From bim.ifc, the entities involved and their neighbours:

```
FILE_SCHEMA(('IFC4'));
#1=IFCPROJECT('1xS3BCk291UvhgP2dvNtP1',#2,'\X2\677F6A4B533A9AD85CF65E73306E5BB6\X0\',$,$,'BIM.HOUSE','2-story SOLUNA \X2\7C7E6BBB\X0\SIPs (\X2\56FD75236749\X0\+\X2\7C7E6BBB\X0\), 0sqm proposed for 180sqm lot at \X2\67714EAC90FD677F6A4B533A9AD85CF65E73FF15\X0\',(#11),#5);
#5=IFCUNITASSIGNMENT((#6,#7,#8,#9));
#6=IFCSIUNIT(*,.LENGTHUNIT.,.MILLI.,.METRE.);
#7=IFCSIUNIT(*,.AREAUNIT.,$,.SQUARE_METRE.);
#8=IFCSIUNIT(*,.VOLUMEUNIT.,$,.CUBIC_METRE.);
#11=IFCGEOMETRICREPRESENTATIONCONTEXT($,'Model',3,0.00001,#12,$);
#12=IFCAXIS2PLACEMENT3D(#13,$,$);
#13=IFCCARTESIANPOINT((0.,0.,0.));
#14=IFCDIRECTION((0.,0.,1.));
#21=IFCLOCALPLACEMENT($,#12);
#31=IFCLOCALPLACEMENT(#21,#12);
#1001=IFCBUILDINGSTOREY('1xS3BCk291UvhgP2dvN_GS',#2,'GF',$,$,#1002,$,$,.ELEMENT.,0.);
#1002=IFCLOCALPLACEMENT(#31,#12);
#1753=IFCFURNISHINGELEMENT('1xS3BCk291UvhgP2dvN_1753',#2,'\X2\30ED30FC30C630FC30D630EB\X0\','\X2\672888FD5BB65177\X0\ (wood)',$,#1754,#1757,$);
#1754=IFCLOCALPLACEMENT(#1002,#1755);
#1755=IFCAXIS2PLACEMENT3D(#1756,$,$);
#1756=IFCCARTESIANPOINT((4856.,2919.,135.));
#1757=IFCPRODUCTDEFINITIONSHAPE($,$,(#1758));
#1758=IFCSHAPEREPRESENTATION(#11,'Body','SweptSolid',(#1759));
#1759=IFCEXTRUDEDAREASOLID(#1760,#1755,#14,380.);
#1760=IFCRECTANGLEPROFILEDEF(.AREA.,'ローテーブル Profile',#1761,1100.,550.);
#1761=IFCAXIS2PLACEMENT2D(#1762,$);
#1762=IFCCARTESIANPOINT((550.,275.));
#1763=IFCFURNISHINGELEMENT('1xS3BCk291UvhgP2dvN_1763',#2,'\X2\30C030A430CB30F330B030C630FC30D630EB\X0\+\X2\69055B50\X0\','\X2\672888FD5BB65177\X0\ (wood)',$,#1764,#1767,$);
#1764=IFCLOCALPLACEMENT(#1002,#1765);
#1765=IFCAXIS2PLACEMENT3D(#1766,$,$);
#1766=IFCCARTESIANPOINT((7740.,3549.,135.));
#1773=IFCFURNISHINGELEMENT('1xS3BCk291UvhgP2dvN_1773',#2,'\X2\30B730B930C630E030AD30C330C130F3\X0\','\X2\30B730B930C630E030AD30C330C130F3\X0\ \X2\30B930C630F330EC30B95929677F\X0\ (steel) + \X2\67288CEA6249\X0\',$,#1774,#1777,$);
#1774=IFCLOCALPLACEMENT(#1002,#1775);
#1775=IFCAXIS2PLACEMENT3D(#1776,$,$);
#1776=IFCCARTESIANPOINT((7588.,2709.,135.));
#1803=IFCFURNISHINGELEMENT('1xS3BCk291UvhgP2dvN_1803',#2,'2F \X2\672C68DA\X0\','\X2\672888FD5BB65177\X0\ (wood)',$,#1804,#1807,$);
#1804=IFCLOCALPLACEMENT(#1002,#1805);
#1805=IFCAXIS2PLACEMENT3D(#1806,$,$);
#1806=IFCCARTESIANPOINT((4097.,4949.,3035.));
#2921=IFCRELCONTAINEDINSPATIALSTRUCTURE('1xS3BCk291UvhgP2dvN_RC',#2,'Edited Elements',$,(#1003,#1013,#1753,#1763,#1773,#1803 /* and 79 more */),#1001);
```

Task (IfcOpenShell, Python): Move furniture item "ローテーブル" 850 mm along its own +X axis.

```python
import ifcopenshell
import ifcopenshell.api.geometry
import ifcopenshell.util.placement
import ifcopenshell.util.unit

model = ifcopenshell.open("bim.ifc")
unit_scale = ifcopenshell.util.unit.calculate_unit_scale(model)

item = model.by_guid("1xS3BCk291UvhgP2dvN_1753")
matrix = ifcopenshell.util.placement.get_local_placement(item.ObjectPlacement)
matrix[:3, 3] += matrix[:3, 0] * 0.85 / unit_scale
ifcopenshell.api.geometry.edit_object_placement(model, product=item, matrix=matrix, is_si=False)

print(ifcopenshell.util.placement.get_local_placement(item.ObjectPlacement).round(3) + 0.0)

model.write("bim_rev.ifc")
```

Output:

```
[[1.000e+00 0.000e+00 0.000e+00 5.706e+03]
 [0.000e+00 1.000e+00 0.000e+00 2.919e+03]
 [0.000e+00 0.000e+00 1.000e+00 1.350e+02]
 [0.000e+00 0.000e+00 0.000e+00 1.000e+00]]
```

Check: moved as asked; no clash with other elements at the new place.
